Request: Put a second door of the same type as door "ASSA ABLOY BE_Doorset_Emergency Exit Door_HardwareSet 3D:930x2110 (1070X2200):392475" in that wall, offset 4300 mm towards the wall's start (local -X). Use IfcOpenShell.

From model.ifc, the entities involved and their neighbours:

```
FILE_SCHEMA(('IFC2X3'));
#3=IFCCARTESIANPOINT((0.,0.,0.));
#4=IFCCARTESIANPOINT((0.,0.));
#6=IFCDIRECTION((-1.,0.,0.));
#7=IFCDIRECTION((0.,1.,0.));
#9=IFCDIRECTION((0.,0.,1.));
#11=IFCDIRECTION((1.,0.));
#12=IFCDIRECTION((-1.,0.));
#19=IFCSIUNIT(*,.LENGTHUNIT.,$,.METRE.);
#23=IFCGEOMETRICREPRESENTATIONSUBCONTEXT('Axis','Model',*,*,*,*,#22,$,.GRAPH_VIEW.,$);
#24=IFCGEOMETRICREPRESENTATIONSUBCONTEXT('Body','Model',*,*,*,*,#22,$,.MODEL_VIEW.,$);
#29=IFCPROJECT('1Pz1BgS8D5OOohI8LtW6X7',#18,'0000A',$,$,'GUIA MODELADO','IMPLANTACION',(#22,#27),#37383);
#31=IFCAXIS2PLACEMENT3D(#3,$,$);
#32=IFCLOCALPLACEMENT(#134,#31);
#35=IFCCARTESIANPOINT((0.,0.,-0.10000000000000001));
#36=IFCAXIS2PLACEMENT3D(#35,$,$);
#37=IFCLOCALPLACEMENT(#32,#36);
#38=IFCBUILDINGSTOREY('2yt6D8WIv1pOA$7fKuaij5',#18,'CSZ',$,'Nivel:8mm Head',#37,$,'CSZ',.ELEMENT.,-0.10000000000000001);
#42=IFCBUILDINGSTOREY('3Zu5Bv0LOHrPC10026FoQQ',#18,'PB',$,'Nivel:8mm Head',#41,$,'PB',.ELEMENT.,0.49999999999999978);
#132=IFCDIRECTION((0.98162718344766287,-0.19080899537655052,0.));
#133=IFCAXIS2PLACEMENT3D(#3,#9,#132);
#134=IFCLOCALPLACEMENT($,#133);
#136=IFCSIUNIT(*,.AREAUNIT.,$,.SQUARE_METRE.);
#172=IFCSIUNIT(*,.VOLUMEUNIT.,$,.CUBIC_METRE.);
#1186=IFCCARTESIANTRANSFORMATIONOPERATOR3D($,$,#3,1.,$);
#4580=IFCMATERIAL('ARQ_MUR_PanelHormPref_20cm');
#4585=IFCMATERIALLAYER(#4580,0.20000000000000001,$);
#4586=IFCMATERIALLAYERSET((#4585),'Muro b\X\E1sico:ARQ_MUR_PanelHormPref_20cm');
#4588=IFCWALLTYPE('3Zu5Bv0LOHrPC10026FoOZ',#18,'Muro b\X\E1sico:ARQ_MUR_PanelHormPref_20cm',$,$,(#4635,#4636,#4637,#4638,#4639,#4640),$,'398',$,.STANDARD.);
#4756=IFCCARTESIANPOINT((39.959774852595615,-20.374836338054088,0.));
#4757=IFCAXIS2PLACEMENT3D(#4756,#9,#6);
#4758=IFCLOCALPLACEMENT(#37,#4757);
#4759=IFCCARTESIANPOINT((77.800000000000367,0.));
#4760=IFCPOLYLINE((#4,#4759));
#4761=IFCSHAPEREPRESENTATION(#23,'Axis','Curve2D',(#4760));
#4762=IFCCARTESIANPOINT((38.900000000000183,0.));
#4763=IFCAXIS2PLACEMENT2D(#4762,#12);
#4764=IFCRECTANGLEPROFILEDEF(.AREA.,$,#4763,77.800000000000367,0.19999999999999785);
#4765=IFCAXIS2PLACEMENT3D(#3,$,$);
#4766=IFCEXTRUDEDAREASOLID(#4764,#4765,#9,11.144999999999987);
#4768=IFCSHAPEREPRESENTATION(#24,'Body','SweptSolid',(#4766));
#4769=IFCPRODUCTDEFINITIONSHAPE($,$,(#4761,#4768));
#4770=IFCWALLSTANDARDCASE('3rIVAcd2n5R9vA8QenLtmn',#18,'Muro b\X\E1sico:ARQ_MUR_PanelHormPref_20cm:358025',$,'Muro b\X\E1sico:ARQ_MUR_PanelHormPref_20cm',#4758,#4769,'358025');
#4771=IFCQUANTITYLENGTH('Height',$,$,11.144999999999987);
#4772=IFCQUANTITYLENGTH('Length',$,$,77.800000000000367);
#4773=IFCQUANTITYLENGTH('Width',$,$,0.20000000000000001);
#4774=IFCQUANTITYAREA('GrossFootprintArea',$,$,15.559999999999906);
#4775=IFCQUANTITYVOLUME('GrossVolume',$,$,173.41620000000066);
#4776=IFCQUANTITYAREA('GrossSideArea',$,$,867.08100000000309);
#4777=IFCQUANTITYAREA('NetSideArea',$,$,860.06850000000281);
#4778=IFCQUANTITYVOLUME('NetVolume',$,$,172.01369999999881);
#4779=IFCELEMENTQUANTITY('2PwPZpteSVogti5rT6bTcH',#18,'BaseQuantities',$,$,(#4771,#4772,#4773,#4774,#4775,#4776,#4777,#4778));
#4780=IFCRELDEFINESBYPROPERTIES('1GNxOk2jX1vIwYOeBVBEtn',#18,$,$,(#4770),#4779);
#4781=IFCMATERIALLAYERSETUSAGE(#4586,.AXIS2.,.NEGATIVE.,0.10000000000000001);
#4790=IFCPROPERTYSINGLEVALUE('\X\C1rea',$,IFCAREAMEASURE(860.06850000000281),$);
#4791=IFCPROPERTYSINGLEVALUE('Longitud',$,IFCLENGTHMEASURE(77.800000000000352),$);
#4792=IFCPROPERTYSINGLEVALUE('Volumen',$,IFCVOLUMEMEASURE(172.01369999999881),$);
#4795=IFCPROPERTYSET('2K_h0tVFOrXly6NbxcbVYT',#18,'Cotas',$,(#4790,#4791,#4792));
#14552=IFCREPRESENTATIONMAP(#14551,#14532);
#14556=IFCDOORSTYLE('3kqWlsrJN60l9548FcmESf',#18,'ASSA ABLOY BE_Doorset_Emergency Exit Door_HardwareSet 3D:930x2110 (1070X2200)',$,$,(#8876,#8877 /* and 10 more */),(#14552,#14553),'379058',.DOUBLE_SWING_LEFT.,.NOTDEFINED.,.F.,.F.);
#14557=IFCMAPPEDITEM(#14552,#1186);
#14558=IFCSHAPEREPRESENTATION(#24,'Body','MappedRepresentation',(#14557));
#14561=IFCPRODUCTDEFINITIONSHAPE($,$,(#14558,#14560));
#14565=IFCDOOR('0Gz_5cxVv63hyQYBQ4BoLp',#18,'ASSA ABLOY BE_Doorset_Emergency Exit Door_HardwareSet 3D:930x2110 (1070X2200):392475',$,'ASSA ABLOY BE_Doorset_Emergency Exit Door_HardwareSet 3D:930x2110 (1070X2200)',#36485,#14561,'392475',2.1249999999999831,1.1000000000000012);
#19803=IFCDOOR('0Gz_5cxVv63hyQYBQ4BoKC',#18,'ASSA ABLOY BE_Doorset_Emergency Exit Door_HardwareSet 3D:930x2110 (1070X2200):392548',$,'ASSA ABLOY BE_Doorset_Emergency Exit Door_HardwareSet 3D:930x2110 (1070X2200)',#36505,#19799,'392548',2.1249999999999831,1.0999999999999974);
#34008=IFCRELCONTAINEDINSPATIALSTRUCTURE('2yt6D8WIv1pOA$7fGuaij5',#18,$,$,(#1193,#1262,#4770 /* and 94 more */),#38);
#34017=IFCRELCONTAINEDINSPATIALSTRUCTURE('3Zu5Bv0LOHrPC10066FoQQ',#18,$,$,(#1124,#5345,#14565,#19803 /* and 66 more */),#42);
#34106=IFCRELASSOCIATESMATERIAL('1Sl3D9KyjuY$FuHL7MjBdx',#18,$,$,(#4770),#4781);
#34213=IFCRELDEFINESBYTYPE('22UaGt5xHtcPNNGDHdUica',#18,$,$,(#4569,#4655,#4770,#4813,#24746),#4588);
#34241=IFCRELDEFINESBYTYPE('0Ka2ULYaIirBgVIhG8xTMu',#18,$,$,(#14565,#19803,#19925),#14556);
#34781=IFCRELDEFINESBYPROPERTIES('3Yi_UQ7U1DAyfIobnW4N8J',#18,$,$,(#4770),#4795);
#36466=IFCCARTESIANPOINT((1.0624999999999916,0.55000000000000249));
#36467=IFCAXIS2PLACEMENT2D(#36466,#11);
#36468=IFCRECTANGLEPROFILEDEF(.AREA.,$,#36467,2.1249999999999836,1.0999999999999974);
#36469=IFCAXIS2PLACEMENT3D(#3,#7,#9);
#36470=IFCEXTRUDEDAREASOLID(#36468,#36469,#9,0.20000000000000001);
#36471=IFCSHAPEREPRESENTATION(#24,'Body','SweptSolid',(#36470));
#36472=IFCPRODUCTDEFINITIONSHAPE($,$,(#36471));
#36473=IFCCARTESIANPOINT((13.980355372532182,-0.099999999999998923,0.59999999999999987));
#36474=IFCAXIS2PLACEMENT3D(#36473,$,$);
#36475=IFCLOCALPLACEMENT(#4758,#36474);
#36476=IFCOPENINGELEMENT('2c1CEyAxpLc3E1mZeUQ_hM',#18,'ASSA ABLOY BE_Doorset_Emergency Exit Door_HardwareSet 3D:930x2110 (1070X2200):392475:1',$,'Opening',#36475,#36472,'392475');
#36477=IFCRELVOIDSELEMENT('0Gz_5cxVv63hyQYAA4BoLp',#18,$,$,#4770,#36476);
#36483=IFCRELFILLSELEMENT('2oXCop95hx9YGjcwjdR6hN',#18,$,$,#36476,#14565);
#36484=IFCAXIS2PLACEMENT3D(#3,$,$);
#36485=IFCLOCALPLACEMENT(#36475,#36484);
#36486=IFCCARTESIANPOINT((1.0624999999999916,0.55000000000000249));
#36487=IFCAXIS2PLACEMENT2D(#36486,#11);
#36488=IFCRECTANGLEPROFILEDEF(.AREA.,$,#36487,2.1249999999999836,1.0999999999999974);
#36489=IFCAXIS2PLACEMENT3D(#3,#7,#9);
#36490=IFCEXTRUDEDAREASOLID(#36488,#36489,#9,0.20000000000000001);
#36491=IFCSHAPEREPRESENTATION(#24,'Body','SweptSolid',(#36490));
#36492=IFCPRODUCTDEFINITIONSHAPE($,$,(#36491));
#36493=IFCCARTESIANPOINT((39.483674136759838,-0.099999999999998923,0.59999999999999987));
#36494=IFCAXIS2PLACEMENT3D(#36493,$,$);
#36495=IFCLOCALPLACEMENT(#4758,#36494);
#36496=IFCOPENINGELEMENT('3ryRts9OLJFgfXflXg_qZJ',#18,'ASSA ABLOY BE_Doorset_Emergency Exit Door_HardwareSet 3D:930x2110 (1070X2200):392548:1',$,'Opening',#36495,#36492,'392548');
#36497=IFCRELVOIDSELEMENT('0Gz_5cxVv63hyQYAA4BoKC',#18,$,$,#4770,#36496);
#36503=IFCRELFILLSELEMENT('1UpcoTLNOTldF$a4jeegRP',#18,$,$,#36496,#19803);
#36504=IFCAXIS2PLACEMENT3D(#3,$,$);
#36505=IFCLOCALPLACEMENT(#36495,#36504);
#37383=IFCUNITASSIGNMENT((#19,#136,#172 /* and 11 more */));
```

```python
import ifcopenshell
import ifcopenshell.api.feature
import ifcopenshell.api.geometry
import ifcopenshell.api.pset
import ifcopenshell.api.root
import ifcopenshell.geom
import ifcopenshell.util.element
import ifcopenshell.util.placement
import ifcopenshell.util.shape
import ifcopenshell.util.unit

model = ifcopenshell.open("model.ifc")
unit_scale = ifcopenshell.util.unit.calculate_unit_scale(model)
area_scale = ifcopenshell.util.unit.calculate_unit_scale(model, "AREAUNIT")
volume_scale = ifcopenshell.util.unit.calculate_unit_scale(model, "VOLUMEUNIT")
settings = ifcopenshell.geom.settings()


def volume(element):
    """Net volume in cubic metres, openings subtracted."""
    shape = ifcopenshell.geom.create_shape(settings, element)
    return ifcopenshell.util.shape.get_volume(shape.geometry)


def reuse_history(source, copy):
    """copy_class also copies each property set's owner history, people and application; keep the originals."""
    for rel in copy.IsDefinedBy:
        if rel.is_a("IfcRelDefinesByProperties") and (history := rel.RelatingPropertyDefinition.OwnerHistory):
            rel.RelatingPropertyDefinition.OwnerHistory = source.OwnerHistory
            ifcopenshell.util.element.remove_deep2(model, history)


door = model.by_guid("0Gz_5cxVv63hyQYBQ4BoLp")
opening = door.FillsVoids[0].RelatingOpeningElement
wall = opening.VoidsElements[0].RelatingBuildingElement
before = volume(wall)
shift = ifcopenshell.util.placement.get_local_placement(wall.ObjectPlacement)[:3, 0] * -4.3 / unit_scale

# copy_class copies the void relationship, type, container and properties, but no geometry.
new_opening = ifcopenshell.api.root.copy_class(model, product=opening)
new_opening.Representation = ifcopenshell.util.element.copy_deep(
    model, opening.Representation, exclude=["IfcGeometricRepresentationContext", "IfcRepresentationMap"]
)
new_opening.Name = "ASSA ABLOY BE_Doorset_Emergency Exit Door_HardwareSet 3D:930x2110 (1070X2200)"
new_opening.Tag = None
reuse_history(opening, new_opening)
new_door = ifcopenshell.api.root.copy_class(model, product=door)
new_door.Representation = ifcopenshell.util.element.copy_deep(
    model, door.Representation, exclude=["IfcGeometricRepresentationContext", "IfcRepresentationMap"]
)
new_door.Name = "ASSA ABLOY BE_Doorset_Emergency Exit Door_HardwareSet 3D:930x2110 (1070X2200)"
new_door.Tag = None
reuse_history(door, new_door)
fills = ifcopenshell.api.feature.add_filling(model, opening=new_opening, element=new_door)
fills.OwnerHistory = new_door.OwnerHistory  # required in IFC2X3

for old, new in ((opening, new_opening), (door, new_door)):
    matrix = ifcopenshell.util.placement.get_local_placement(old.ObjectPlacement)
    matrix[:3, 3] += shift
    ifcopenshell.api.geometry.edit_object_placement(model, product=new, matrix=matrix, is_si=False)

after = volume(wall)
thickness = 0.2  # wall thickness in metres

# Update the wall's stored quantities.
qto = model.by_id(ifcopenshell.util.element.get_pset(wall, "BaseQuantities", should_inherit=False)["id"])
ifcopenshell.api.pset.edit_qto(model, qto=qto, properties={
    "NetSideArea": after / thickness / area_scale,
    "NetVolume": after / volume_scale,
})
pset = model.by_id(ifcopenshell.util.element.get_pset(wall, "Cotas", should_inherit=False)["id"])
ifcopenshell.api.pset.edit_pset(model, pset=pset, properties={
    "Área": model.create_entity("IfcAreaMeasure", after / thickness / area_scale),
    "Volumen": model.create_entity("IfcVolumeMeasure", after / volume_scale),
})

print(f"wall volume {before:.3f} -> {after:.3f} m3")

model.write("model-out.ifc")
```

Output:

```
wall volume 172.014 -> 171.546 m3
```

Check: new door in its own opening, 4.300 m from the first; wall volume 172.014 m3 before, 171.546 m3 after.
